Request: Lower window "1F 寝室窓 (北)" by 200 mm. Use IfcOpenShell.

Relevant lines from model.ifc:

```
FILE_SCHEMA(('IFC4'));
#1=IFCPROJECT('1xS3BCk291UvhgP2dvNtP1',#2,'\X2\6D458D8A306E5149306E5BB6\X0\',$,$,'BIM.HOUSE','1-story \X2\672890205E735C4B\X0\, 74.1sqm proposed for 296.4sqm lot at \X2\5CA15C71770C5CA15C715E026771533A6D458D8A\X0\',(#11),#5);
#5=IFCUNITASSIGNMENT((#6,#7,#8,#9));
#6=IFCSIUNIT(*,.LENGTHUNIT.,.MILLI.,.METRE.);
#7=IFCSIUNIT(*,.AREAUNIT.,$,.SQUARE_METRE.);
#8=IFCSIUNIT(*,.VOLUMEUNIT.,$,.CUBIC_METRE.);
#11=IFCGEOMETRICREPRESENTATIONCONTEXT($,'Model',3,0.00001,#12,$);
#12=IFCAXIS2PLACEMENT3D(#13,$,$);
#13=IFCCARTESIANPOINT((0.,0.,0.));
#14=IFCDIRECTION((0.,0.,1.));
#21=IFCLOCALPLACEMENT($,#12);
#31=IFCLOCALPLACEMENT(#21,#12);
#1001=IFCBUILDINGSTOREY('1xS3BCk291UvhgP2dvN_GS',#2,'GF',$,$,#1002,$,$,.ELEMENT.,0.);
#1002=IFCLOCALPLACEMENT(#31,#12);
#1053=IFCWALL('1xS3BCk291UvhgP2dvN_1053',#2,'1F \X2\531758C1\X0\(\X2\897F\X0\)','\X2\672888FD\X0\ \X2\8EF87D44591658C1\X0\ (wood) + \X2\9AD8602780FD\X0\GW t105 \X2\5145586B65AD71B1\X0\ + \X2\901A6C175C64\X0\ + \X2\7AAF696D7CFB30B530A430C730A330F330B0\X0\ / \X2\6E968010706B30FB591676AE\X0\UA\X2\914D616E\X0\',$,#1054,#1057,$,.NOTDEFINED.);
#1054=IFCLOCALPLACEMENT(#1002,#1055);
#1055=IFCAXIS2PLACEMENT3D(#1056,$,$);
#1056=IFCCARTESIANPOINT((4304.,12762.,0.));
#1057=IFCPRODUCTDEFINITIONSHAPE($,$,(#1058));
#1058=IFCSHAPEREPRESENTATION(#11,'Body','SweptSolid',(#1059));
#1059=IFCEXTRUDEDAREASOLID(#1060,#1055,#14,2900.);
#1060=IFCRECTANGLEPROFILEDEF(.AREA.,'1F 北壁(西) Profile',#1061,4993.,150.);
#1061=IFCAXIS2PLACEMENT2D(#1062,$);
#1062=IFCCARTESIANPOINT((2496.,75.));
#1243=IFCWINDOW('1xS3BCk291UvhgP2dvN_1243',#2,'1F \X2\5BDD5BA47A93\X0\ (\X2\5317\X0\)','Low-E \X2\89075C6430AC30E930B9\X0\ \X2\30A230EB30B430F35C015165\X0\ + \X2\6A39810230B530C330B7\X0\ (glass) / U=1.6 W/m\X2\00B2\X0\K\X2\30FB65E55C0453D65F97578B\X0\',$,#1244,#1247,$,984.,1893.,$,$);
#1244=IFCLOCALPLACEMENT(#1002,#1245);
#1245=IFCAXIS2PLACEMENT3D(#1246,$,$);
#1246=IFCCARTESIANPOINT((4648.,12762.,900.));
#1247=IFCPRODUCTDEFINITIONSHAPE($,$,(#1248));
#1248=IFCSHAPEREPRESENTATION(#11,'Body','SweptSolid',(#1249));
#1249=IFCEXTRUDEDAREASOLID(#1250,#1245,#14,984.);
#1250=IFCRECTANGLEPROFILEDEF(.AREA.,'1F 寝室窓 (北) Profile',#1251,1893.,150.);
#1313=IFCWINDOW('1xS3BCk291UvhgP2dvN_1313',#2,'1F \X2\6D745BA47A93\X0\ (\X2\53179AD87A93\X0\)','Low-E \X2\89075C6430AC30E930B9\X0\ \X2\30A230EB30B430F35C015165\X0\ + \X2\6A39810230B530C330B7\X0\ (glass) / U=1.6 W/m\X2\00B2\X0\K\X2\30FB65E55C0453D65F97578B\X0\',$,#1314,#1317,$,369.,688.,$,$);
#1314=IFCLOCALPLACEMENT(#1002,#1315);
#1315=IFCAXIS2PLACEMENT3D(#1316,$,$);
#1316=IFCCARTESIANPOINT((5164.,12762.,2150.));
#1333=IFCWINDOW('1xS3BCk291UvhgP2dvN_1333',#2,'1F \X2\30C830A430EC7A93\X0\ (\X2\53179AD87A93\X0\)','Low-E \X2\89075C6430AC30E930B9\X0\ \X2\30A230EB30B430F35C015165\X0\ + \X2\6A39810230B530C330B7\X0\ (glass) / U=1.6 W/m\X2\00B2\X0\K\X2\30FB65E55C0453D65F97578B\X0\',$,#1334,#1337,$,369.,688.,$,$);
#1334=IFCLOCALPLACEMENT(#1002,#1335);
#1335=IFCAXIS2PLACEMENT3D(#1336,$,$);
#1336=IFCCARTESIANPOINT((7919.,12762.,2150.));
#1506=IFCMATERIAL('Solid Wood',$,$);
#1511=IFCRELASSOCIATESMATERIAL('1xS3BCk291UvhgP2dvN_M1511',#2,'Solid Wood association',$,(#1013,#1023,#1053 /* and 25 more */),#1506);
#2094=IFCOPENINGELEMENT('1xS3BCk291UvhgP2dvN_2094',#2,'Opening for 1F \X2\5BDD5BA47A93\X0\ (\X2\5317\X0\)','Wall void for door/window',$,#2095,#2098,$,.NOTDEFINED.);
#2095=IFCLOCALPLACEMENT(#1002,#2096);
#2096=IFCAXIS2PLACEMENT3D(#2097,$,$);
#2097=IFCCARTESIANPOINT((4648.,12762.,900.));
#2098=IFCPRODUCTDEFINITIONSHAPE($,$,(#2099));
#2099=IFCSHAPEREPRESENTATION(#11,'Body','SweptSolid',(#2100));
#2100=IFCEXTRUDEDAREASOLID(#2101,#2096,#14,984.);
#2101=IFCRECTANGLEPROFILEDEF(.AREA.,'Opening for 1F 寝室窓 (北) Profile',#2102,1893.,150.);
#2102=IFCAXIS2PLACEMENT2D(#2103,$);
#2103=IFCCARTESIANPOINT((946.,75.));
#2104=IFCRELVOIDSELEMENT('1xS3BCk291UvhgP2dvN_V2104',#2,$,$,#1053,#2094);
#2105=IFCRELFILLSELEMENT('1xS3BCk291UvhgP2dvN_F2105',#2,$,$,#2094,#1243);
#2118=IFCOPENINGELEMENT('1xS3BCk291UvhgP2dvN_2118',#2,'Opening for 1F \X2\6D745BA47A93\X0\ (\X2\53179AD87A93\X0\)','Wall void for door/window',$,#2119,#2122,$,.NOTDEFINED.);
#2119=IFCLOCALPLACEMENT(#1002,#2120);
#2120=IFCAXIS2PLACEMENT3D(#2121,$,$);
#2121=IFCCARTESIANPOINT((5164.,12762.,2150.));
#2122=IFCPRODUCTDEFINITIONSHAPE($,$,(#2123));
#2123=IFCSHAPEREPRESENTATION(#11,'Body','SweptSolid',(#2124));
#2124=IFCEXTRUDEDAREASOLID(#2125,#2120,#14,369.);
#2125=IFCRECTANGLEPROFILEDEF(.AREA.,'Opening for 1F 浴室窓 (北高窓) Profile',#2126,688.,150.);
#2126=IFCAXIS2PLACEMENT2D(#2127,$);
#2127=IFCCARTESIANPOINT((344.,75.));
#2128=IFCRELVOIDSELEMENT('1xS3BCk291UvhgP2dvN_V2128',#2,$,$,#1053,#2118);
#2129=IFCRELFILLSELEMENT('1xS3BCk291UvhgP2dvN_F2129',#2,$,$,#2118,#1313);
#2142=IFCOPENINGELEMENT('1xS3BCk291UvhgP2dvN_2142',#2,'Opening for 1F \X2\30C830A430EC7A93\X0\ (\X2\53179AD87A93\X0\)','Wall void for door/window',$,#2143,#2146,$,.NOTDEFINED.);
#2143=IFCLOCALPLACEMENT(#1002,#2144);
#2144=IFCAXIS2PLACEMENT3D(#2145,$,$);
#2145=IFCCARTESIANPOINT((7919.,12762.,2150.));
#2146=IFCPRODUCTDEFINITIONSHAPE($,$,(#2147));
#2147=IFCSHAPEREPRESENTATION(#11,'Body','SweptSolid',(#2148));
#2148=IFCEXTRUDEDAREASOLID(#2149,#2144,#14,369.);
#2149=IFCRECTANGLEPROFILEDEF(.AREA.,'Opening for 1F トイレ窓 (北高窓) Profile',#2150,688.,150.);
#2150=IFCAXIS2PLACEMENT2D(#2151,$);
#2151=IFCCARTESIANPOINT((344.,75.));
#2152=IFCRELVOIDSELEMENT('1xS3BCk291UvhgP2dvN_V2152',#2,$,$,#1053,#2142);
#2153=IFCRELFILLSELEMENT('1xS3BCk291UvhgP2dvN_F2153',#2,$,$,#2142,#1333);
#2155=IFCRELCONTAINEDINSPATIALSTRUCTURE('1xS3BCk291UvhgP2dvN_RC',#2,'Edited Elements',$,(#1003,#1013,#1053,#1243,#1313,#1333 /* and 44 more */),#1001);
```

```python
import numpy as np
import ifcopenshell
import ifcopenshell.api.geometry
import ifcopenshell.util.placement
import ifcopenshell.util.unit

model = ifcopenshell.open("model.ifc")
unit_scale = ifcopenshell.util.unit.calculate_unit_scale(model)

window = model.by_id(1243)
opening = window.FillsVoids[0].RelatingOpeningElement
dz = -0.2 / unit_scale

shift = np.array([0.0, 0.0, dz])
# The window is not placed relative to its opening, so move both.
for product in (opening, window):
    matrix = ifcopenshell.util.placement.get_local_placement(product.ObjectPlacement)
    matrix[:3, 3] += shift
    ifcopenshell.api.geometry.edit_object_placement(model, product=product, matrix=matrix, is_si=False)

print(f"moved by {dz * unit_scale:+.3f} m")

model.write("model_v2.ifc")
```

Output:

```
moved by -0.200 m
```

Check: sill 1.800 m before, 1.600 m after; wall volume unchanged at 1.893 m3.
